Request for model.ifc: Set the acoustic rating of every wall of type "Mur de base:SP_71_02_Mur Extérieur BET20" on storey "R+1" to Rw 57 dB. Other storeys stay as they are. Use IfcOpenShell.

First a look at what the model holds.

```python
import ifcopenshell
import ifcopenshell.util.element

model = ifcopenshell.open("model.ifc")
print(model.schema)
storey = next(s for s in model.by_type("IfcBuildingStorey") if s.Name == "R+1")
walls = [e for e in ifcopenshell.util.element.get_decomposition(storey) if e.is_a("IfcWall")]
seen = {}
for e in walls:
    element_type = ifcopenshell.util.element.get_type(e)
    key = (element_type.Name if element_type != e and element_type else None, ifcopenshell.util.element.get_pset(e, "Pset_WallCommon", "AcousticRating"))
    seen[key] = seen.get(key, 0) + 1
for (name, value), count in sorted(seen.items(), key=str):
    print(count, "x", name, "|", value)
```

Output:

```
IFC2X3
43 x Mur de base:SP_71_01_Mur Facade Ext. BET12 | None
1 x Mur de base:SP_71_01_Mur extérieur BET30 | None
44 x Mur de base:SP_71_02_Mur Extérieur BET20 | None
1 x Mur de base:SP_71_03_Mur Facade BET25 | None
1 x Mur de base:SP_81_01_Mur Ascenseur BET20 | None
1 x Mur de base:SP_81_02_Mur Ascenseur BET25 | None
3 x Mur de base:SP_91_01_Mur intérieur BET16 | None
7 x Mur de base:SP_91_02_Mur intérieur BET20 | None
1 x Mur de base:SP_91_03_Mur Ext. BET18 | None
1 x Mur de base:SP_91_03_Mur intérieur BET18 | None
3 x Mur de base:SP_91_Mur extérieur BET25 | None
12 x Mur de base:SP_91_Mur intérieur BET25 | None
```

```python
import ifcopenshell
import ifcopenshell.api.pset
import ifcopenshell.util.element

model = ifcopenshell.open("model.ifc")

storey = next(s for s in model.by_type("IfcBuildingStorey") if s.Name == "R+1")
walls = [e for e in ifcopenshell.util.element.get_decomposition(storey) if e.is_a("IfcWall")]

count = 0
for e in walls:
    element_type = ifcopenshell.util.element.get_type(e)
    if element_type in (None, e) or element_type.Name != "Mur de base:SP_71_02_Mur Extérieur BET20":
        continue
    found = ifcopenshell.util.element.get_pset(e, "Pset_WallCommon", should_inherit=False)
    if found:
        pset = model.by_id(found["id"])
        if len(ifcopenshell.util.element.get_elements_by_pset(pset)) > 1:
            pset = ifcopenshell.api.pset.unshare_pset(model, products=[e], pset=pset)[0]
    else:
        pset = ifcopenshell.api.pset.add_pset(model, product=e, name="Pset_WallCommon")
    ifcopenshell.api.pset.edit_pset(model, pset=pset, properties={"AcousticRating": "Rw 57 dB"})
    count += 1

print(count, "walls updated")

model.write("model_updated.ifc")
```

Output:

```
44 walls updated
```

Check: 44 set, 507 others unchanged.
